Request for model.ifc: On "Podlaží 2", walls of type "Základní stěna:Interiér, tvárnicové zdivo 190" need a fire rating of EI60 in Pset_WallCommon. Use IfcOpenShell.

First a look at what the model holds.

```python
import ifcopenshell
import ifcopenshell.util.element

model = ifcopenshell.open("model.ifc")
print(model.schema)
storey = next(s for s in model.by_type("IfcBuildingStorey") if s.Name == "Podlaží 2")
walls = [e for e in ifcopenshell.util.element.get_decomposition(storey) if e.is_a("IfcWall")]
seen = {}
for e in walls:
    element_type = ifcopenshell.util.element.get_type(e)
    key = (element_type.Name if element_type != e and element_type else None, ifcopenshell.util.element.get_pset(e, "Pset_WallCommon", "FireRating"))
    seen[key] = seen.get(key, 0) + 1
for (name, value), count in sorted(seen.items(), key=str):
    print(count, "x", name, "|", value)
```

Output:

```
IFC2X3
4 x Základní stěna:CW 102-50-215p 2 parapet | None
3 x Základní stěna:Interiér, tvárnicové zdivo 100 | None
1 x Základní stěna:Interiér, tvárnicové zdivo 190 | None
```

```python
import ifcopenshell
import ifcopenshell.api.pset
import ifcopenshell.util.element

model = ifcopenshell.open("model.ifc")

storey = next(s for s in model.by_type("IfcBuildingStorey") if s.Name == "Podlaží 2")
walls = [e for e in ifcopenshell.util.element.get_decomposition(storey) if e.is_a("IfcWall")]

count = 0
for e in walls:
    element_type = ifcopenshell.util.element.get_type(e)
    if element_type in (None, e) or element_type.Name != "Základní stěna:Interiér, tvárnicové zdivo 190":
        continue
    # add_pset returns the element's existing set when there is one.
    pset = ifcopenshell.api.pset.add_pset(model, product=e, name="Pset_WallCommon")
    ifcopenshell.api.pset.edit_pset(model, pset=pset, properties={"FireRating": "EI60"})
    count += 1

print(count, "walls updated")

model.write("model_v2.ifc")
```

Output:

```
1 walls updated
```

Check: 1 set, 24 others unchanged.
